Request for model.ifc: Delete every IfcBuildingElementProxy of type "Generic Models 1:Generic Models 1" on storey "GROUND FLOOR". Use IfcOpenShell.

First a look at what the model holds.

```python
import ifcopenshell
import ifcopenshell.util.element

model = ifcopenshell.open("model.ifc")
print(model.schema)
storey = next(s for s in model.by_type("IfcBuildingStorey") if s.Name == "GROUND FLOOR")
proxies = [e for e in ifcopenshell.util.element.get_decomposition(storey) if e.is_a("IfcBuildingElementProxy")]
seen = {}
for e in proxies:
    element_type = ifcopenshell.util.element.get_type(e)
    name = element_type.Name if element_type not in (None, e) else None
    seen[name] = seen.get(name, 0) + 1
for name, count in sorted(seen.items(), key=str):
    print(count, "x", name)
```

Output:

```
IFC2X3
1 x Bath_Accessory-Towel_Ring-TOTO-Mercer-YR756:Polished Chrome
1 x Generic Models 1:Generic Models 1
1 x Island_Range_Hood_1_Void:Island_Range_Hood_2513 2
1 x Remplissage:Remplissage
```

```python
import ifcopenshell
import ifcopenshell.api.root
import ifcopenshell.util.element

model = ifcopenshell.open("model.ifc")

storey = next(s for s in model.by_type("IfcBuildingStorey") if s.Name == "GROUND FLOOR")
proxies = [e for e in ifcopenshell.util.element.get_decomposition(storey) if e.is_a("IfcBuildingElementProxy")]
targets = [e for e in proxies if (t := ifcopenshell.util.element.get_type(e)) not in (None, e) and t.Name == "Generic Models 1:Generic Models 1"]

for e in targets:
    ifcopenshell.api.root.remove_product(model, product=e)
print(len(targets), "removed")

model.write("model-out.ifc")
```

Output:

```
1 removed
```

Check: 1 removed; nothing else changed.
